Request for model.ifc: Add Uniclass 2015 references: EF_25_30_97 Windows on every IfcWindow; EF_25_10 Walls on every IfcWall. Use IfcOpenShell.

First a look at what the model holds.

```python
import ifcopenshell

model = ifcopenshell.open("model.ifc")
print(model.schema)
print("classifications:", [c.Name for c in model.by_type("IfcClassification")])
for ifc_class in ("IfcDoor", "IfcRoof", "IfcStair", "IfcWall", "IfcWindow"):
    print(ifc_class, len(model.by_type(ifc_class)))
```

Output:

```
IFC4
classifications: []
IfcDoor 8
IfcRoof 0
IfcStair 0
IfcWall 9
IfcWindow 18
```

```python
import ifcopenshell
import ifcopenshell.api.classification

model = ifcopenshell.open("model.ifc")

system = ifcopenshell.api.classification.add_classification(model, classification="Uniclass 2015")

codes = {
    "IfcWindow": ("EF_25_30_97", "Windows"),
    "IfcWall": ("EF_25_10", "Walls"),
}
for ifc_class, (code, name) in codes.items():
    products = model.by_type(ifc_class)
    ifcopenshell.api.classification.add_reference(
        model, products=products, classification=system, identification=code, name=name
    )
    print(code, len(products))

model.write("model_v2.ifc")
```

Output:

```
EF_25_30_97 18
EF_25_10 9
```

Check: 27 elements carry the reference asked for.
